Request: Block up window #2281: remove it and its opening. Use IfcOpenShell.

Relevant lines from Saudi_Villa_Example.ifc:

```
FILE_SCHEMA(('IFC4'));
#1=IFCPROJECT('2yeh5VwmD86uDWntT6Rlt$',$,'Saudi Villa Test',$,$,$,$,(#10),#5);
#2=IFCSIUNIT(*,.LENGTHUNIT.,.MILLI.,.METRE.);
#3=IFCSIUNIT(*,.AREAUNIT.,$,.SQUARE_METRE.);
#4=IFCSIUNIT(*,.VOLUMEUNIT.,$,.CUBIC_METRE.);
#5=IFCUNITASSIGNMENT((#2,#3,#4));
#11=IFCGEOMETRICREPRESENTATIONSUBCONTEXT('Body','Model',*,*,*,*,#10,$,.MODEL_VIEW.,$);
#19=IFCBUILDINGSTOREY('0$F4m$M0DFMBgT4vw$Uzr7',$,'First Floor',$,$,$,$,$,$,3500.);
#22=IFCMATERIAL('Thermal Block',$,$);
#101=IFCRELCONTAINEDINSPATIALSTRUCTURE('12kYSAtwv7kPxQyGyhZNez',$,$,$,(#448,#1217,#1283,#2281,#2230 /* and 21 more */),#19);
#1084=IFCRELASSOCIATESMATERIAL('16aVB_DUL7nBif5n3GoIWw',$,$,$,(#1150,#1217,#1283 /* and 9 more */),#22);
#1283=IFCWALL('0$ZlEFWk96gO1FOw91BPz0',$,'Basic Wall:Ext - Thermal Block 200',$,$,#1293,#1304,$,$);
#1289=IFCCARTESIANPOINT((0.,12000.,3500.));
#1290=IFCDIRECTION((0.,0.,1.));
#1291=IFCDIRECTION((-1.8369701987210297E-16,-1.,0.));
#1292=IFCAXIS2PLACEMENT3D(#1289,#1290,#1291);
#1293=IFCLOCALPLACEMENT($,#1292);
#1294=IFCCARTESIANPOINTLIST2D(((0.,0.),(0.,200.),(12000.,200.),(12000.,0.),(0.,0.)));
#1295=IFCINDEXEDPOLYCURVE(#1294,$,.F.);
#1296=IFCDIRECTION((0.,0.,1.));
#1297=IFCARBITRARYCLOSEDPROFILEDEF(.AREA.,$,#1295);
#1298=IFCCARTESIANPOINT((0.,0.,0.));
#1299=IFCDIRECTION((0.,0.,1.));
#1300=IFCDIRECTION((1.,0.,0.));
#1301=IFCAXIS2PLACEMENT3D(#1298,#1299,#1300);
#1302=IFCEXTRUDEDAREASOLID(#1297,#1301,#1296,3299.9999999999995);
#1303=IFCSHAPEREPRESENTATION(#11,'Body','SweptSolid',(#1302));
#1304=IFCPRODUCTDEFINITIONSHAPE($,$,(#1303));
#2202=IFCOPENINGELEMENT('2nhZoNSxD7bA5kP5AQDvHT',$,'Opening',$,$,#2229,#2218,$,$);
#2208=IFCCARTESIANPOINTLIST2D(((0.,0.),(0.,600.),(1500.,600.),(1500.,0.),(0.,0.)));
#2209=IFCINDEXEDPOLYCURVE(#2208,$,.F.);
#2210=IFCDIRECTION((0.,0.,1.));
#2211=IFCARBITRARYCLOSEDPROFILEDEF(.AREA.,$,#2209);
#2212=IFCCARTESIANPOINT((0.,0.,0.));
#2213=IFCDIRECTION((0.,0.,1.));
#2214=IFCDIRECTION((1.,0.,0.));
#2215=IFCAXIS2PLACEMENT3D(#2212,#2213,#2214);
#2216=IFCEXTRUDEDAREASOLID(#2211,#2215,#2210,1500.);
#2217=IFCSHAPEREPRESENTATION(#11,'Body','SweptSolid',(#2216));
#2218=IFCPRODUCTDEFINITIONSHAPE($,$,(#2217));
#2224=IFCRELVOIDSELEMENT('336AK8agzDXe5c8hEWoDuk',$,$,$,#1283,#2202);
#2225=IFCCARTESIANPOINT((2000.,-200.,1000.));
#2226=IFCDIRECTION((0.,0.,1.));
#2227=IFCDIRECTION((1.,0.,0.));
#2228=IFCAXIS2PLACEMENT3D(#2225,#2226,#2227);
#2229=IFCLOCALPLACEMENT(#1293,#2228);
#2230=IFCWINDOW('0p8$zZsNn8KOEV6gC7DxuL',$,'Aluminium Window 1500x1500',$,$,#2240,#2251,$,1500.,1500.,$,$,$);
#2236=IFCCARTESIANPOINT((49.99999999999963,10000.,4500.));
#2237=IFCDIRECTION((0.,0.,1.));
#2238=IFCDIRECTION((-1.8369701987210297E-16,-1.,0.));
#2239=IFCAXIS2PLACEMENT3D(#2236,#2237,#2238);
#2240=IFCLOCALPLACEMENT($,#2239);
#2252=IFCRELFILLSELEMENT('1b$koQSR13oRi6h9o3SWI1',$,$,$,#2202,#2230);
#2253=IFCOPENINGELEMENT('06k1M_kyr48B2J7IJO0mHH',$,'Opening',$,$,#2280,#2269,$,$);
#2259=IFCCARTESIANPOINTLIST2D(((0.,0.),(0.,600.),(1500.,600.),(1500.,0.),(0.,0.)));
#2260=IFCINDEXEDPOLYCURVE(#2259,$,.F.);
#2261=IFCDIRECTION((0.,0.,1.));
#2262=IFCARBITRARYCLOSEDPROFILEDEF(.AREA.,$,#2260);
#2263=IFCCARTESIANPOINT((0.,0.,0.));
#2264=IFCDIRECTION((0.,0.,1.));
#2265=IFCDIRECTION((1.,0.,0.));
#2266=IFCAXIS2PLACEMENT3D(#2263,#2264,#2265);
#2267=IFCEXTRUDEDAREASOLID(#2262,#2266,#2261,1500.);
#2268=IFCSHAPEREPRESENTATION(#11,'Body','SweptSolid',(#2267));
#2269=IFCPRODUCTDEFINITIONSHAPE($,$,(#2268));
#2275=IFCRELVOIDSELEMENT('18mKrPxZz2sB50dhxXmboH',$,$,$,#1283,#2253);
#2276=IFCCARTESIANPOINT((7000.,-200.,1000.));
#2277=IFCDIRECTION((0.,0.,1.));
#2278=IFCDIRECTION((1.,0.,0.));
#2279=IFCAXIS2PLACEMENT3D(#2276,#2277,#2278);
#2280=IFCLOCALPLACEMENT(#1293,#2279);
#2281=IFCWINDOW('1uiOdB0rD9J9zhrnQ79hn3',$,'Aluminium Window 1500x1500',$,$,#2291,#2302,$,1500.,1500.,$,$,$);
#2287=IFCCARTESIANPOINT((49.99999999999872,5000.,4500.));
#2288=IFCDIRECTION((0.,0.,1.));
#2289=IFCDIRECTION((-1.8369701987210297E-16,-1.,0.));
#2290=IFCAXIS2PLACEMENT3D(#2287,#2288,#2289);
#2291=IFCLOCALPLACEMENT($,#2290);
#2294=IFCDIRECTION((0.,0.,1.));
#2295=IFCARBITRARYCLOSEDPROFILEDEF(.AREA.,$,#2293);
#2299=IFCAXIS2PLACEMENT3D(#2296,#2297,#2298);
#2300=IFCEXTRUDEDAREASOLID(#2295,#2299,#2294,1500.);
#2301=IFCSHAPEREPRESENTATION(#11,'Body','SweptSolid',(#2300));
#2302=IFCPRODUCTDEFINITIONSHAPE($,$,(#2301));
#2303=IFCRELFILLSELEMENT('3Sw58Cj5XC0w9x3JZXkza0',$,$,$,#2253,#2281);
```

```python
import ifcopenshell
import ifcopenshell.api.feature
import ifcopenshell.api.root
import ifcopenshell.geom
import ifcopenshell.util.shape

model = ifcopenshell.open("Saudi_Villa_Example.ifc")
settings = ifcopenshell.geom.settings()


def volume(element):
    """Net volume in cubic metres, openings subtracted."""
    shape = ifcopenshell.geom.create_shape(settings, element)
    return ifcopenshell.util.shape.get_volume(shape.geometry)


window = model.by_guid("1uiOdB0rD9J9zhrnQ79hn3")
opening = window.FillsVoids[0].RelatingOpeningElement
wall = opening.VoidsElements[0].RelatingBuildingElement
before = volume(wall)

ifcopenshell.api.root.remove_product(model, product=window)
ifcopenshell.api.feature.remove_feature(model, feature=opening)

after = volume(wall)

print(f"wall volume {before:.3f} -> {after:.3f} m3")

model.write("Saudi_Villa_Example-out.ifc")
```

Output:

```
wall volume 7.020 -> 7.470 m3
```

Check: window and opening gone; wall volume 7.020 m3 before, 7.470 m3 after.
